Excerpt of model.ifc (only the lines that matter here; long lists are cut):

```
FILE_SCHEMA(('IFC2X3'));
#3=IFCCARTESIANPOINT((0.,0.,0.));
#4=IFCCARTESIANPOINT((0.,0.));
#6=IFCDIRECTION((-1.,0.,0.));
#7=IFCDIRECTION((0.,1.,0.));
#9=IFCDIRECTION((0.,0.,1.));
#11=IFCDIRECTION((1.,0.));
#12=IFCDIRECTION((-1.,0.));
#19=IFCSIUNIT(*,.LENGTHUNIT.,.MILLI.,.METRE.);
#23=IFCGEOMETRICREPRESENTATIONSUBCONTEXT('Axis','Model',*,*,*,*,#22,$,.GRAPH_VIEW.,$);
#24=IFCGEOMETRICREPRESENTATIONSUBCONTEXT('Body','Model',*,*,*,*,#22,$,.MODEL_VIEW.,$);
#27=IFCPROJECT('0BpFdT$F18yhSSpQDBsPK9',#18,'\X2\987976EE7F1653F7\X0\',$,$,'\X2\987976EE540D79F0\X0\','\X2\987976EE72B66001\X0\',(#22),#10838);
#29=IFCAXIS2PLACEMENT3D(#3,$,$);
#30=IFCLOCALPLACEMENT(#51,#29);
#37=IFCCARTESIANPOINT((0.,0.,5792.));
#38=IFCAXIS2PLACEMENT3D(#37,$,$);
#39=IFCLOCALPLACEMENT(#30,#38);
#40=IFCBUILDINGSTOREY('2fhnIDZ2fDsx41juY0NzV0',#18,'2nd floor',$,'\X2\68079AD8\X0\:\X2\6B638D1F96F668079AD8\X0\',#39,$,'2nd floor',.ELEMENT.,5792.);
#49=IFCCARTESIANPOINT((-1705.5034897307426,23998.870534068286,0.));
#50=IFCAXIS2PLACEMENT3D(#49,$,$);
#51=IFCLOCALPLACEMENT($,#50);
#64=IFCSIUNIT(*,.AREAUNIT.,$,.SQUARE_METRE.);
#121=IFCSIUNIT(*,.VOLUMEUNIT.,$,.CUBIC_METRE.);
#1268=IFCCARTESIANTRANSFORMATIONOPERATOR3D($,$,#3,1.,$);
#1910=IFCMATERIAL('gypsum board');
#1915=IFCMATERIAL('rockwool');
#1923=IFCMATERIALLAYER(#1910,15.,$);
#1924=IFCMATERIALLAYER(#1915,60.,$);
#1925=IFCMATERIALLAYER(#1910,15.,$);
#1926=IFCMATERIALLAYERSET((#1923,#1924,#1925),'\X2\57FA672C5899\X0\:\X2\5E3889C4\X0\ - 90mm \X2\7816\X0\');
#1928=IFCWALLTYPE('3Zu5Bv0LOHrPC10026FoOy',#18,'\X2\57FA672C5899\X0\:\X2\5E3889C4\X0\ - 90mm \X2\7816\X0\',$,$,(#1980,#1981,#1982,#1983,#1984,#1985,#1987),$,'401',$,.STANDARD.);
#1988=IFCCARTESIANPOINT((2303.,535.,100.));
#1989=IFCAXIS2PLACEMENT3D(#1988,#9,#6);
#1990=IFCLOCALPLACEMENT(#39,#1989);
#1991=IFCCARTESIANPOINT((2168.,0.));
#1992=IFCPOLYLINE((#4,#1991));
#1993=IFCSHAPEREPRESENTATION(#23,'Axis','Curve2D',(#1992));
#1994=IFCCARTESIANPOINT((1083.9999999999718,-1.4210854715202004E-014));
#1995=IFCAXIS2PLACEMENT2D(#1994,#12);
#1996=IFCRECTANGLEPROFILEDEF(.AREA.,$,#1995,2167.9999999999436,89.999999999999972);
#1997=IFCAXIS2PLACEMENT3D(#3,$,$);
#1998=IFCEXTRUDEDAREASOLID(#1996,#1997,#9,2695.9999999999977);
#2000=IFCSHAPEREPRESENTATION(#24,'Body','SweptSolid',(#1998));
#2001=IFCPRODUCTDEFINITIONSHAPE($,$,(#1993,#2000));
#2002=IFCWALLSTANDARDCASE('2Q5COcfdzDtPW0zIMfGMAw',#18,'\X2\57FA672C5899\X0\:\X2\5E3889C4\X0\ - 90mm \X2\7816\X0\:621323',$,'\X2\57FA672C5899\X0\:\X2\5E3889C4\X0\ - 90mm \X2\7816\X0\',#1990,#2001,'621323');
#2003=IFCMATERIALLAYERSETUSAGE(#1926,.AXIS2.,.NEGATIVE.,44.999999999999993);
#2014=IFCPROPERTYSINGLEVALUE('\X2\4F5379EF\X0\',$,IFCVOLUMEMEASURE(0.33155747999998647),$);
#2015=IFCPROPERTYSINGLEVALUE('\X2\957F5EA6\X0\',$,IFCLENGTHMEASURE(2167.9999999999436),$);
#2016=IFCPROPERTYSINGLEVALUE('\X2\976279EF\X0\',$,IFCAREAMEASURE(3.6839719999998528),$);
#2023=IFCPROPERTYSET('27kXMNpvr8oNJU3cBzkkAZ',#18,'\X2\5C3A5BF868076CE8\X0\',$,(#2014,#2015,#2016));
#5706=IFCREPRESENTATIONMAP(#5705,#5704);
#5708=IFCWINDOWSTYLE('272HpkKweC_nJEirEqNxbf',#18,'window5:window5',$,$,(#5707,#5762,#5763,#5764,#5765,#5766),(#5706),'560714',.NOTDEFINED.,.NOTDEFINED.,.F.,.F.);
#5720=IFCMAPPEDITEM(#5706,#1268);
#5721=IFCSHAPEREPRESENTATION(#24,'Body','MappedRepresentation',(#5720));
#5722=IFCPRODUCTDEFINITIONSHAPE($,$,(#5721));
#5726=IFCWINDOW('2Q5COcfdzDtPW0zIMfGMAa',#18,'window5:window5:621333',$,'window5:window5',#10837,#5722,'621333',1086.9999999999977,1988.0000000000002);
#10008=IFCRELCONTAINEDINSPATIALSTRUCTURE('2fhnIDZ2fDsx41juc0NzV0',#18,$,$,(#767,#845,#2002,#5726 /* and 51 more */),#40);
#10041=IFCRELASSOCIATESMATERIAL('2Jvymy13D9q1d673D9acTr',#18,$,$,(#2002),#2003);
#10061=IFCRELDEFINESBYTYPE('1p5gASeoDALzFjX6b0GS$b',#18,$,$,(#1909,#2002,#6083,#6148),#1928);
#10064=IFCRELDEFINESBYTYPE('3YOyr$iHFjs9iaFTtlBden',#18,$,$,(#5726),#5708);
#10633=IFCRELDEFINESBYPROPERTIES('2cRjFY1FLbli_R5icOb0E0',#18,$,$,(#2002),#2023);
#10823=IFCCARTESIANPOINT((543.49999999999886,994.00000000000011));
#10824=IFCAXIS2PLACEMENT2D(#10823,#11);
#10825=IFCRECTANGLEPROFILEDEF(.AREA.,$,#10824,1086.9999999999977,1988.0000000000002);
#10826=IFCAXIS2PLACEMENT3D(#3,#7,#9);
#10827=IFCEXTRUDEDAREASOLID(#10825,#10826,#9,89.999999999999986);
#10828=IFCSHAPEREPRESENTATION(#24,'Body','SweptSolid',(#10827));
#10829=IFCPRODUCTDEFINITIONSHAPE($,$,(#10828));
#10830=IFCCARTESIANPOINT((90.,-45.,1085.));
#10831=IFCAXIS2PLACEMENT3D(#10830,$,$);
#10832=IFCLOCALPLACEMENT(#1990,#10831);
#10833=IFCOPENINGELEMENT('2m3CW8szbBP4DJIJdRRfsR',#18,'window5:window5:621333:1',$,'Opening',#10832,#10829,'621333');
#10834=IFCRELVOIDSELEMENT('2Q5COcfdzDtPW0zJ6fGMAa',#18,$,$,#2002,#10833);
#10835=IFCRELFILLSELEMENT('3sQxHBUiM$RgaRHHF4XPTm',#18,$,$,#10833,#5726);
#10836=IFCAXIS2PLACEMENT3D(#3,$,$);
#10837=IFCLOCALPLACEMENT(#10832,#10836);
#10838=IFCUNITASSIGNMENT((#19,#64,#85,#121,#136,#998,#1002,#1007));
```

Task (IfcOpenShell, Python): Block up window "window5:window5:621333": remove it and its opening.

```python
import ifcopenshell
import ifcopenshell.api.feature
import ifcopenshell.api.pset
import ifcopenshell.api.root
import ifcopenshell.geom
import ifcopenshell.util.element
import ifcopenshell.util.shape
import ifcopenshell.util.unit

model = ifcopenshell.open("model.ifc")
area_scale = ifcopenshell.util.unit.calculate_unit_scale(model, "AREAUNIT")
volume_scale = ifcopenshell.util.unit.calculate_unit_scale(model, "VOLUMEUNIT")
settings = ifcopenshell.geom.settings()


def volume(element):
    """Net volume in cubic metres, openings subtracted."""
    shape = ifcopenshell.geom.create_shape(settings, element)
    return ifcopenshell.util.shape.get_volume(shape.geometry)


window = model.by_id(5726)
opening = window.FillsVoids[0].RelatingOpeningElement
wall = opening.VoidsElements[0].RelatingBuildingElement
before = volume(wall)

ifcopenshell.api.root.remove_product(model, product=window)
ifcopenshell.api.feature.remove_feature(model, feature=opening)

after = volume(wall)
thickness = 0.09  # wall thickness in metres

# Update the wall's stored quantities.
pset = model.by_id(ifcopenshell.util.element.get_pset(wall, "尺寸标注", should_inherit=False)["id"])
ifcopenshell.api.pset.edit_pset(model, pset=pset, properties={
    "体积": model.create_entity("IfcVolumeMeasure", after / volume_scale),
    "面积": model.create_entity("IfcAreaMeasure", after / thickness / area_scale),
})

print(f"wall volume {before:.3f} -> {after:.3f} m3")

model.write("model_updated.ifc")
```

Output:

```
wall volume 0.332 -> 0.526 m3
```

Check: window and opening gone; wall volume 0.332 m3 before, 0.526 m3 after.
